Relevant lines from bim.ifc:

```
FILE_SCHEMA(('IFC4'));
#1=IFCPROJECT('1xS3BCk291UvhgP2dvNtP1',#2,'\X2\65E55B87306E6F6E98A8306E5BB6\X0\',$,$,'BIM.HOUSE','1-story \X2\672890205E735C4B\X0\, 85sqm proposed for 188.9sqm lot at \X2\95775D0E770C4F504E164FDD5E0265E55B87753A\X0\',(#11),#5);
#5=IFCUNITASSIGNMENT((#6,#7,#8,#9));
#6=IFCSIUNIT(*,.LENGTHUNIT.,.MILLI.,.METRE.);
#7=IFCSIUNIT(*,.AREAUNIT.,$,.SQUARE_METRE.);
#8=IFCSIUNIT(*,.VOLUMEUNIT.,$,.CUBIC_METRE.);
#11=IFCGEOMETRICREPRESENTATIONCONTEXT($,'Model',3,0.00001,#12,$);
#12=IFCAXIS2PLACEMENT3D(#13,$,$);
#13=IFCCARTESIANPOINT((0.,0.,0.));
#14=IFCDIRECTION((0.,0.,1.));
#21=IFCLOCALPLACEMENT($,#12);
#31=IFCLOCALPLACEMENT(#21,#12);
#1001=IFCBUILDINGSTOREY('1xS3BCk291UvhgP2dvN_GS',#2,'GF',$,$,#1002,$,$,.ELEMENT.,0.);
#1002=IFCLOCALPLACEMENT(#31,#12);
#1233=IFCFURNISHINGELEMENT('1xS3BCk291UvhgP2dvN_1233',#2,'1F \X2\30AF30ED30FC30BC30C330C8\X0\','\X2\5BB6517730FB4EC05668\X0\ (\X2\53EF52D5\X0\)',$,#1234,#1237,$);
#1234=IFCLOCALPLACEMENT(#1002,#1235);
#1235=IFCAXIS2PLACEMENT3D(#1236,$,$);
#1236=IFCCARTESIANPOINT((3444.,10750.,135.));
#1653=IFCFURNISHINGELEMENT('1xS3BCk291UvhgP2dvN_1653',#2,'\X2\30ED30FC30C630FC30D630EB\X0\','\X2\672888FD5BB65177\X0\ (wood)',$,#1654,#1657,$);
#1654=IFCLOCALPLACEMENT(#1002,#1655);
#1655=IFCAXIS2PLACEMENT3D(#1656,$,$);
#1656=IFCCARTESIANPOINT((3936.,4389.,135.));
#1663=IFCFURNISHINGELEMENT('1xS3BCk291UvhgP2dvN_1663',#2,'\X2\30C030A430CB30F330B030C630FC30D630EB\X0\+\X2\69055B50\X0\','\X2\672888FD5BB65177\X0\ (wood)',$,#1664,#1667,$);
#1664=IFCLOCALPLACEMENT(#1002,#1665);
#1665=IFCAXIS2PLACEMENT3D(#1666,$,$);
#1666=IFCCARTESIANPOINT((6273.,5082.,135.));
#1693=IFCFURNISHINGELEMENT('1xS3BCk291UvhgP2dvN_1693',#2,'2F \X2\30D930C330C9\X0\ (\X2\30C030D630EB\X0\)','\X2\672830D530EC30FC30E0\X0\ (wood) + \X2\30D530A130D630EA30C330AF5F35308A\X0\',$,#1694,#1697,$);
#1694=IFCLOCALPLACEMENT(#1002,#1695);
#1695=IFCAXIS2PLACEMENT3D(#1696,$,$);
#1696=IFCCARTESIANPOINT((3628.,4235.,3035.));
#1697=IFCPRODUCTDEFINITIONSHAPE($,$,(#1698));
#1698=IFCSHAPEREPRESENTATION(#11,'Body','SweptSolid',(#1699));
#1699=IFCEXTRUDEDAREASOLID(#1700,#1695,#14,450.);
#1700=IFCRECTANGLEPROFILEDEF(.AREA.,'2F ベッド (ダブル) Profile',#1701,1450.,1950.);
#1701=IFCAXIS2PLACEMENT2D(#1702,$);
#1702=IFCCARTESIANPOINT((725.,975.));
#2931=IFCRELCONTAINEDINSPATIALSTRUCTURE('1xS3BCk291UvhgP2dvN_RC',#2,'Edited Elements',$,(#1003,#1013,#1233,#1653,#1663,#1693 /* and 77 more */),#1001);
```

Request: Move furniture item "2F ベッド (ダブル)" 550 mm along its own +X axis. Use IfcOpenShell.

```python
import ifcopenshell
import ifcopenshell.api.geometry
import ifcopenshell.util.placement
import ifcopenshell.util.unit

model = ifcopenshell.open("bim.ifc")
unit_scale = ifcopenshell.util.unit.calculate_unit_scale(model)

item = model.by_guid("1xS3BCk291UvhgP2dvN_1693")
matrix = ifcopenshell.util.placement.get_local_placement(item.ObjectPlacement)
matrix[:3, 3] += matrix[:3, 0] * 0.55 / unit_scale
ifcopenshell.api.geometry.edit_object_placement(model, product=item, matrix=matrix, is_si=False)

print(ifcopenshell.util.placement.get_local_placement(item.ObjectPlacement).round(3) + 0.0)

model.write("bim_rev.ifc")
```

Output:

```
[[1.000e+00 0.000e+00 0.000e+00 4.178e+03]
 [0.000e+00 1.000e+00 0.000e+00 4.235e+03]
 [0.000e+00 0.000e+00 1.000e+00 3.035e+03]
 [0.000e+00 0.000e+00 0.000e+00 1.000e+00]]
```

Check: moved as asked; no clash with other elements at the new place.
